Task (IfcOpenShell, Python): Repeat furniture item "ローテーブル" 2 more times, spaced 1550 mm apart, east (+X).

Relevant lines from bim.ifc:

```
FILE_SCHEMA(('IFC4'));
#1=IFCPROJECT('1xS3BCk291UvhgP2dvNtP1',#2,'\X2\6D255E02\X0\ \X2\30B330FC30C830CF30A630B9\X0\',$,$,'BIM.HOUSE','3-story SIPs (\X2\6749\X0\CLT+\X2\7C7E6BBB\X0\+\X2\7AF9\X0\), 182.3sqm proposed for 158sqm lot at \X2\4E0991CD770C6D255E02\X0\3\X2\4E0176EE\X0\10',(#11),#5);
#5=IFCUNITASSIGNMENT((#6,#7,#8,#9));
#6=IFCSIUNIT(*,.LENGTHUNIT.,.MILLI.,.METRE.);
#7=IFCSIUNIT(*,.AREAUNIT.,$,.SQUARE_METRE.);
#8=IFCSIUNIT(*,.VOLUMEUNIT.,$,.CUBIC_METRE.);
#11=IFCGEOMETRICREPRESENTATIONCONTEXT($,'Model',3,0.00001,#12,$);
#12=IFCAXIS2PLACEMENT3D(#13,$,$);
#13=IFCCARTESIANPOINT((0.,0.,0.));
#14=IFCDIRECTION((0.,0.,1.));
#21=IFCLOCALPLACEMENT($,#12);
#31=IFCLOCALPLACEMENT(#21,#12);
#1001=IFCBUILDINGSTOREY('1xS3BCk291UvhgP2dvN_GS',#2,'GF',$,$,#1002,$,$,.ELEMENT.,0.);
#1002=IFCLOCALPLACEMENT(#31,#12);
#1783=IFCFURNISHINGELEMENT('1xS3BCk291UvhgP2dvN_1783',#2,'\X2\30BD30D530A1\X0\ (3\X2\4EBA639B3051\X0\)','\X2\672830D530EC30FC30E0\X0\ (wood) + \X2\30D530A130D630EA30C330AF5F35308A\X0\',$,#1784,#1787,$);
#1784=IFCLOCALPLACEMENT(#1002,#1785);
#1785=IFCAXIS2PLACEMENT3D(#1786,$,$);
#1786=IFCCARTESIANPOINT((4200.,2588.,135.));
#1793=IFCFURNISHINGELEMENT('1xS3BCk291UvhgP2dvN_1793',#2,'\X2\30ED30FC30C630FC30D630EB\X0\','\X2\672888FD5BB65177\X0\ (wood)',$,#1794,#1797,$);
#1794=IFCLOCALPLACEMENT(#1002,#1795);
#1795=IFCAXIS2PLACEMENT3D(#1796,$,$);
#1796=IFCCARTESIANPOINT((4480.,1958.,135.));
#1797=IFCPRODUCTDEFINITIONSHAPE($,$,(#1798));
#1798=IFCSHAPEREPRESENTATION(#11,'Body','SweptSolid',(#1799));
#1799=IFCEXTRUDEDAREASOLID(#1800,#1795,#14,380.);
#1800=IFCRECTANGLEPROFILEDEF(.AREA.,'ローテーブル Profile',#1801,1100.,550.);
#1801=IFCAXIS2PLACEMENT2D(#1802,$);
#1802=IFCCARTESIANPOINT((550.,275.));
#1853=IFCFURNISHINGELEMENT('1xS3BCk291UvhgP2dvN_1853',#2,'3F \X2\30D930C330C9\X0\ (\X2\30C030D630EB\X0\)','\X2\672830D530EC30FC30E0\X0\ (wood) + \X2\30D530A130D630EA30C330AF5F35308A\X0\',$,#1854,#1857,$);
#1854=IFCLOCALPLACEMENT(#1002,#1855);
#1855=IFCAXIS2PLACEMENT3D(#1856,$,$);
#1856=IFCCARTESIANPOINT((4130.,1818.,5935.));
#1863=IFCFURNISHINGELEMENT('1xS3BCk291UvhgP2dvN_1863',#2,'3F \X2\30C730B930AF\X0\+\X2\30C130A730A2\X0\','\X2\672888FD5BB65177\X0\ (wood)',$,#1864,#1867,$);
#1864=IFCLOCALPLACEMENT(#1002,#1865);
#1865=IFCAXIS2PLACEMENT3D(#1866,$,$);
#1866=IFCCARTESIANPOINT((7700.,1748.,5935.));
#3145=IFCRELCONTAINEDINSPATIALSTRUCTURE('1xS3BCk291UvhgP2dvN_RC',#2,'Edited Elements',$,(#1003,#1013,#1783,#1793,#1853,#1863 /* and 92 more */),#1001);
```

```python
import numpy as np
import ifcopenshell
import ifcopenshell.api.geometry
import ifcopenshell.api.root
import ifcopenshell.util.element
import ifcopenshell.util.placement
import ifcopenshell.util.unit

model = ifcopenshell.open("bim.ifc")
unit_scale = ifcopenshell.util.unit.calculate_unit_scale(model)


def reuse_history(source, copy):
    """copy_class also copies each property set's owner history, people and application; keep the originals."""
    for rel in copy.IsDefinedBy:
        if rel.is_a("IfcRelDefinesByProperties") and (history := rel.RelatingPropertyDefinition.OwnerHistory):
            rel.RelatingPropertyDefinition.OwnerHistory = source.OwnerHistory
            ifcopenshell.util.element.remove_deep2(model, history)


source = model.by_id(1793)
base = ifcopenshell.util.placement.get_local_placement(source.ObjectPlacement)
step = np.array([1.0, 0.0, 0.0]) * 1.55 / unit_scale

for i in range(1, 3):
    copy = ifcopenshell.api.root.copy_class(model, product=source)
    copy.Representation = ifcopenshell.util.element.copy_deep(
        model, source.Representation, exclude=["IfcGeometricRepresentationContext", "IfcRepresentationMap"]
    )
    reuse_history(source, copy)
    matrix = base.copy()
    matrix[:3, 3] += i * step
    print("added at", matrix[:3, 3].round(3) + 0.0)
    ifcopenshell.api.geometry.edit_object_placement(model, product=copy, matrix=matrix, is_si=False)

model.write("bim_edited.ifc")
```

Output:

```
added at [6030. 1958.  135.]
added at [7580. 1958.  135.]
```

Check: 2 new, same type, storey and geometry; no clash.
